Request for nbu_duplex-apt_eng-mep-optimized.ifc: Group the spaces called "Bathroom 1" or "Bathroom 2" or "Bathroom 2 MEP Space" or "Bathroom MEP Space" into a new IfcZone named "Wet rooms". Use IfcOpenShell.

First a look at what the model holds.

```python
import ifcopenshell

model = ifcopenshell.open("nbu_duplex-apt_eng-mep-optimized.ifc")
print(model.schema)
seen = {}
for space in model.by_type("IfcSpace"):
    seen[space.LongName] = seen.get(space.LongName, 0) + 1
for name, count in sorted(seen.items(), key=str):
    print(count, "x", name)
print("zones:", [z.Name for z in model.by_type("IfcZone")][:20])
```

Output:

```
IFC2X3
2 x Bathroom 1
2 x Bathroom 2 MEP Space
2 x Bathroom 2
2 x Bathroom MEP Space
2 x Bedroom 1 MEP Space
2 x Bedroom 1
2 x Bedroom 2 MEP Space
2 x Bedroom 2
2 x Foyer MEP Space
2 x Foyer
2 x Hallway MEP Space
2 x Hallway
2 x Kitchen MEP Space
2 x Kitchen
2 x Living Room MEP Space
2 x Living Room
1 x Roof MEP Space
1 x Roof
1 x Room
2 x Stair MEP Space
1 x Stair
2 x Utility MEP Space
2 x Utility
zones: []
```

```python
import ifcopenshell
import ifcopenshell.api.group
import ifcopenshell.api.root

model = ifcopenshell.open("nbu_duplex-apt_eng-mep-optimized.ifc")

names = {"Bathroom 1", "Bathroom 2", "Bathroom 2 MEP Space", "Bathroom MEP Space"}
spaces = [s for s in model.by_type("IfcSpace") if s.LongName in names]

zone = ifcopenshell.api.root.create_entity(model, ifc_class="IfcZone", name="Wet rooms")
ifcopenshell.api.group.assign_group(model, products=spaces, group=zone)
print(len(spaces), "spaces in", zone.Name)

model.write("nbu_duplex-apt_eng-mep-optimized_edited.ifc")
```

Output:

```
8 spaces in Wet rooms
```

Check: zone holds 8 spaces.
